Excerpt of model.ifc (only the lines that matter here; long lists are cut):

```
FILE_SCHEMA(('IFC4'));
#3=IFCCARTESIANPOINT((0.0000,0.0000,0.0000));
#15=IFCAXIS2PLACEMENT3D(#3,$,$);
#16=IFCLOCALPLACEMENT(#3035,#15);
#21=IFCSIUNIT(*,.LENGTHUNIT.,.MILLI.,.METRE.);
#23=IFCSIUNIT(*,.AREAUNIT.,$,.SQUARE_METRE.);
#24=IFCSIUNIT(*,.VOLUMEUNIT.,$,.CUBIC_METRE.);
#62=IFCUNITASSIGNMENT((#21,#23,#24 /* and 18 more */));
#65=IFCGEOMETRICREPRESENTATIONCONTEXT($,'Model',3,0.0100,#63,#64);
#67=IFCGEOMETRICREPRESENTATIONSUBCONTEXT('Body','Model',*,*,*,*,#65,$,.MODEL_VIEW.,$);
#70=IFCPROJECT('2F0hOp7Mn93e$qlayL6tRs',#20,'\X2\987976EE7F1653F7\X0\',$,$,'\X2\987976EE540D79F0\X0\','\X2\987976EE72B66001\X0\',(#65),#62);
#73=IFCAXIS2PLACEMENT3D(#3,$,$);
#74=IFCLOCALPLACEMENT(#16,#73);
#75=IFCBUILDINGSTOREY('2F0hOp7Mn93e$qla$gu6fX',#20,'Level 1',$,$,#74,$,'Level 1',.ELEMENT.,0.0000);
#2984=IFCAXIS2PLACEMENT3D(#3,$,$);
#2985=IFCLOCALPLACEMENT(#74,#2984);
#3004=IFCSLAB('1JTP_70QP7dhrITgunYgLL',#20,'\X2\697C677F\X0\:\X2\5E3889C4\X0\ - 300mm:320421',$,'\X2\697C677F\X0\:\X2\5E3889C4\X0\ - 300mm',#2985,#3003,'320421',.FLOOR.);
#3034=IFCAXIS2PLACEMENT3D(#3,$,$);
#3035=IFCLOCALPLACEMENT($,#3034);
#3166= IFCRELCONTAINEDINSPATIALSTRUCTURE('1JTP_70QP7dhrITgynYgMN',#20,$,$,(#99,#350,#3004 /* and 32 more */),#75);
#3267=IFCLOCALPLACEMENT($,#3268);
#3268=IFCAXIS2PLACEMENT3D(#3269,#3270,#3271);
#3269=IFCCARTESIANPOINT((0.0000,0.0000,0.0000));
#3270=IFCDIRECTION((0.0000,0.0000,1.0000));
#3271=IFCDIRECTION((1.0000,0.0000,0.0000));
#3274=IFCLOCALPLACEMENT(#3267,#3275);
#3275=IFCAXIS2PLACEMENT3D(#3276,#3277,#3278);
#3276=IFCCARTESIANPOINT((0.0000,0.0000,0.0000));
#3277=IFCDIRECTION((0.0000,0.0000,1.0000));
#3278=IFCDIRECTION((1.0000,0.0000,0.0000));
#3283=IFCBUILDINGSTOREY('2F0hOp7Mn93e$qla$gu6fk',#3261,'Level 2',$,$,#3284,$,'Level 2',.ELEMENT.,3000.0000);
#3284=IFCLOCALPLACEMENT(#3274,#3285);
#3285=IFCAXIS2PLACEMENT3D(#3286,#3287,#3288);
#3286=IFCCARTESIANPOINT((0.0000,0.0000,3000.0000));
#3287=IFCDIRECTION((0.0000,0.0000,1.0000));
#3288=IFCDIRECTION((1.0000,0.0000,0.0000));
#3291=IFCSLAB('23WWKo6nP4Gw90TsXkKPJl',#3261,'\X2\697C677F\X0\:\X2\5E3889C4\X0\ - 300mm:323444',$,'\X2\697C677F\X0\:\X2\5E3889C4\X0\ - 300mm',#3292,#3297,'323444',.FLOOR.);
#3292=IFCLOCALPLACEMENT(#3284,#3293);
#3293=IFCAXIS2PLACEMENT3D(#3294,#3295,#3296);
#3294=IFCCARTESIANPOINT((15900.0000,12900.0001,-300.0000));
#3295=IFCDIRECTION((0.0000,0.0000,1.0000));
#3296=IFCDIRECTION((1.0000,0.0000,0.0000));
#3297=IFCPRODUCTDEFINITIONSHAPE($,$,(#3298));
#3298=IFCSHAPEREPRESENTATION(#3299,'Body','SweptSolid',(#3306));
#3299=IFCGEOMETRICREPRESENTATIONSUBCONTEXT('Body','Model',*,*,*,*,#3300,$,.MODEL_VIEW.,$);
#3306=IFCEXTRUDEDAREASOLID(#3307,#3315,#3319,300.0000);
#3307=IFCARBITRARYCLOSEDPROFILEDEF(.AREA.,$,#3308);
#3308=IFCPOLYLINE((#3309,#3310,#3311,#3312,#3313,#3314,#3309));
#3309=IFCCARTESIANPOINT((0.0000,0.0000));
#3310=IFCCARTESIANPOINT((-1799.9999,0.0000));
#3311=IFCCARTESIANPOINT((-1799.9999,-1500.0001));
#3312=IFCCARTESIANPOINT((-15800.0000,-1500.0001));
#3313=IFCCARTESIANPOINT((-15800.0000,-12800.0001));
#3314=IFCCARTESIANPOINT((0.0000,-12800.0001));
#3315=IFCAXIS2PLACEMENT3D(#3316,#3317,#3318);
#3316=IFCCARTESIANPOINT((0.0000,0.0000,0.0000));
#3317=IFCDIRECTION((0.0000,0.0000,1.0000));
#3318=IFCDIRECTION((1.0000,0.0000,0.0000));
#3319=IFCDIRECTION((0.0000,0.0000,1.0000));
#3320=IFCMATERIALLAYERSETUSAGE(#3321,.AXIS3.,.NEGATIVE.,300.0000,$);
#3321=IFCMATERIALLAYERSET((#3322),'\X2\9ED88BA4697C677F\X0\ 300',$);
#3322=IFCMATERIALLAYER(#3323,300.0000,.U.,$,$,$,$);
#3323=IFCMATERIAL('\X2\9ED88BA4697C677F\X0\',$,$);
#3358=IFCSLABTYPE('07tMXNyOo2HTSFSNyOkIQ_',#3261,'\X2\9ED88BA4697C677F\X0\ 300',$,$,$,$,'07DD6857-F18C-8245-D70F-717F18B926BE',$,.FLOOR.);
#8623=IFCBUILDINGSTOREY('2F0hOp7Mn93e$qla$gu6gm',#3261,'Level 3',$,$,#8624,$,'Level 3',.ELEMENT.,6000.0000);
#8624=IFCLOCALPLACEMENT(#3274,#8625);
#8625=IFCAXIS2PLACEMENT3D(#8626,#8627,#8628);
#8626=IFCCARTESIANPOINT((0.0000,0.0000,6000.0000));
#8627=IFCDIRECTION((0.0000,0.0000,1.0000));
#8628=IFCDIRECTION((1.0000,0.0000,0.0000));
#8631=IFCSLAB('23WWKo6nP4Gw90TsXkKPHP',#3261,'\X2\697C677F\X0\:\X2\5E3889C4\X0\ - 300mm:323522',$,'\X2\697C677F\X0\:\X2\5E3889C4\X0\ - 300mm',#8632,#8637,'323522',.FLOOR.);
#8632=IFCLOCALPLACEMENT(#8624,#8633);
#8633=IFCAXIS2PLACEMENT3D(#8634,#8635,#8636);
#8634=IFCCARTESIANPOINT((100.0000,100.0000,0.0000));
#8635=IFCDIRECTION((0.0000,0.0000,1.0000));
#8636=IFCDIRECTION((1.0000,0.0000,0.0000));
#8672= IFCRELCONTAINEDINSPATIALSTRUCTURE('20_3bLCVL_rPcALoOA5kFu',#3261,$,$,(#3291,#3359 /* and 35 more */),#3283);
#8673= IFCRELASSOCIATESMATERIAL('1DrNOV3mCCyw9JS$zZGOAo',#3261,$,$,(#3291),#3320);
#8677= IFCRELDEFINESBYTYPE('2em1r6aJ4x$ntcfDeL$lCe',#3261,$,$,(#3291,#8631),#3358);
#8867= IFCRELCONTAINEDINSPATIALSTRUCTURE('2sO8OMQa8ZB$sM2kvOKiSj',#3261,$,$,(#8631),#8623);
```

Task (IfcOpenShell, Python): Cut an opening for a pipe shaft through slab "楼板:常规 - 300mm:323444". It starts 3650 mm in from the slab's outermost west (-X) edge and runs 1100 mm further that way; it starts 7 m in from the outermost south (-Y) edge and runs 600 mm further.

```python
import numpy as np
import ifcopenshell
import ifcopenshell.api.feature
import ifcopenshell.api.geometry
import ifcopenshell.api.root
import ifcopenshell.geom
import ifcopenshell.util.placement
import ifcopenshell.util.representation
import ifcopenshell.util.shape
import ifcopenshell.util.unit

model = ifcopenshell.open("model.ifc")
unit_scale = ifcopenshell.util.unit.calculate_unit_scale(model)
settings = ifcopenshell.geom.settings()


def volume(element):
    """Net volume in cubic metres, openings subtracted."""
    shape = ifcopenshell.geom.create_shape(settings, element)
    return ifcopenshell.util.shape.get_volume(shape.geometry)


slab = model.by_id(3291)
before = volume(slab)

# Extent in the slab's own axes, in metres. The edges named are its -X and -Y sides.
slab_shape = ifcopenshell.geom.create_shape(settings, slab)
vertices = ifcopenshell.util.shape.get_vertices(slab_shape.geometry)
x_min, y_min, bottom = vertices.min(axis=0)
top = vertices[:, 2].max()

opening = ifcopenshell.api.root.create_entity(model, ifc_class="IfcOpeningElement", name="Pipe shaft opening", predefined_type="OPENING")
context = ifcopenshell.util.representation.get_context(model, "Model", "Body", "MODEL_VIEW")
width, depth = 1.1, 0.6
outline = [(0.0, 0.0), (width, 0.0), (width, depth), (0.0, depth), (0.0, 0.0)]
# Overshoot both faces by 50 mm so the cut is clean.
shape = ifcopenshell.api.geometry.add_slab_representation(
    model, context=context, depth=top - bottom + 0.1, polyline=outline
)
ifcopenshell.api.geometry.assign_representation(model, product=opening, representation=shape)

matrix = ifcopenshell.util.placement.get_local_placement(slab.ObjectPlacement)
matrix[:, 3] = matrix @ np.append(np.array([x_min + 3.65, y_min + 7, bottom - 0.05]) / unit_scale, 1.0)
ifcopenshell.api.geometry.edit_object_placement(model, product=opening, matrix=matrix, is_si=False)
ifcopenshell.api.feature.add_feature(model, feature=opening, element=slab)

after = volume(slab)

print(f"slab volume {before:.3f} -> {after:.3f} m3")

model.write("model-out.ifc")
```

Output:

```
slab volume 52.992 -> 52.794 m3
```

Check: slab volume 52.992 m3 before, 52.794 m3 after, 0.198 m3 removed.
